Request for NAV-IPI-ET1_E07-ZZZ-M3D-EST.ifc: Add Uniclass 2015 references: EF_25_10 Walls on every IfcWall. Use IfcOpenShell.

First a look at what the model holds.

```python
import ifcopenshell

model = ifcopenshell.open("NAV-IPI-ET1_E07-ZZZ-M3D-EST.ifc")
print(model.schema)
print("classifications:", [c.Name for c in model.by_type("IfcClassification")])
for ifc_class in ("IfcDoor", "IfcRoof", "IfcStair", "IfcWall", "IfcWindow"):
    print(ifc_class, len(model.by_type(ifc_class)))
```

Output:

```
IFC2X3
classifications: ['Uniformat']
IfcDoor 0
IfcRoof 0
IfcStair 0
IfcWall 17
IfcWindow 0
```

```python
import ifcopenshell
import ifcopenshell.api.classification

model = ifcopenshell.open("NAV-IPI-ET1_E07-ZZZ-M3D-EST.ifc")

# IFC2X3 requires Source and Edition and has no link from the project to the system.
system = model.create_entity("IfcClassification", Source="NBS", Edition="2015", Name="Uniclass 2015")

codes = {
    "IfcWall": ("EF_25_10", "Walls"),
}
for ifc_class, (code, name) in codes.items():
    products = model.by_type(ifc_class)
    ifcopenshell.api.classification.add_reference(
        model, products=products, classification=system, identification=code, name=name
    )
    print(code, len(products))

model.write("NAV-IPI-ET1_E07-ZZZ-M3D-EST_edited.ifc")
```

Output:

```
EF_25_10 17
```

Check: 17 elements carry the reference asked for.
